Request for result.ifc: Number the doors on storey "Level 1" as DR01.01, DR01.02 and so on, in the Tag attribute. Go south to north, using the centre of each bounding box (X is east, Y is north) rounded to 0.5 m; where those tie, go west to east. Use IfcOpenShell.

First a look at what the model holds.

```python
import ifcopenshell
import ifcopenshell.util.element
import ifcopenshell.util.placement

model = ifcopenshell.open("result.ifc")
print(model.schema)
storey = next(s for s in model.by_type("IfcBuildingStorey") if s.Name == "Level 1")
doors = [e for e in ifcopenshell.util.element.get_decomposition(storey) if e.is_a("IfcDoor")]
for e in sorted(doors, key=lambda e: e.id()):
    origin = ifcopenshell.util.placement.get_local_placement(e.ObjectPlacement)[:3, 3]
    print(e.id(), e.Tag, e.Name, origin.round(2) + 0.0, sep=" | ")
```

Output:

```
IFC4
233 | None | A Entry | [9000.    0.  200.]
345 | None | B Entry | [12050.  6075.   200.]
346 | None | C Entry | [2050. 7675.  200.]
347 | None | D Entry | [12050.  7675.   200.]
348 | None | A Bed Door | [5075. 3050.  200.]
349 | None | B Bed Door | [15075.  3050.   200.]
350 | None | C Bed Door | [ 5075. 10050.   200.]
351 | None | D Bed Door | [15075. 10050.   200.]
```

```python
import ifcopenshell
import ifcopenshell.geom
import ifcopenshell.util.element
import ifcopenshell.util.shape

model = ifcopenshell.open("result.ifc")
settings = ifcopenshell.geom.settings()
settings.set("use-world-coords", True)


def centre(element):
    shape = ifcopenshell.geom.create_shape(settings, element)
    return ifcopenshell.util.shape.get_bbox_centroid(shape.geometry)


storey = next(s for s in model.by_type("IfcBuildingStorey") if s.Name == "Level 1")
doors = [e for e in ifcopenshell.util.element.get_decomposition(storey) if e.is_a("IfcDoor")]

# Insertion points can sit at a corner or the storey origin, so sort by the geometry (in metres).
centres = {e: centre(e) for e in doors}
doors.sort(key=lambda e: (round(centres[e][1] / 0.5), centres[e][0]))

for i, e in enumerate(doors, start=1):
    number = f"DR01.{i:02d}"
    e.Tag = number
    print(e.id(), number)

model.write("result_updated.ifc")
```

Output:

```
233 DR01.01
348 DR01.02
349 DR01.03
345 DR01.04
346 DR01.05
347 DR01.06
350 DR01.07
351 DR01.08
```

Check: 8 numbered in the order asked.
